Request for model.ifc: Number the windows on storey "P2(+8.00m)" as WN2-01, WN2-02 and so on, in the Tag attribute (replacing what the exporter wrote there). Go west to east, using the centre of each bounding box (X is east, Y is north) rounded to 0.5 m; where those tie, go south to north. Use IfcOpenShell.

First a look at what the model holds.

```python
import ifcopenshell
import ifcopenshell.util.element
import ifcopenshell.util.placement

model = ifcopenshell.open("model.ifc")
print(model.schema)
storey = next(s for s in model.by_type("IfcBuildingStorey") if s.Name == "P2(+8.00m)")
windows = [e for e in ifcopenshell.util.element.get_decomposition(storey) if e.is_a("IfcWindow")]
for e in sorted(windows, key=lambda e: e.id()):
    origin = ifcopenshell.util.placement.get_local_placement(e.ObjectPlacement)[:3, 3]
    print(e.id(), e.Tag, e.Name, origin.round(2) + 0.0, sep=" | ")
```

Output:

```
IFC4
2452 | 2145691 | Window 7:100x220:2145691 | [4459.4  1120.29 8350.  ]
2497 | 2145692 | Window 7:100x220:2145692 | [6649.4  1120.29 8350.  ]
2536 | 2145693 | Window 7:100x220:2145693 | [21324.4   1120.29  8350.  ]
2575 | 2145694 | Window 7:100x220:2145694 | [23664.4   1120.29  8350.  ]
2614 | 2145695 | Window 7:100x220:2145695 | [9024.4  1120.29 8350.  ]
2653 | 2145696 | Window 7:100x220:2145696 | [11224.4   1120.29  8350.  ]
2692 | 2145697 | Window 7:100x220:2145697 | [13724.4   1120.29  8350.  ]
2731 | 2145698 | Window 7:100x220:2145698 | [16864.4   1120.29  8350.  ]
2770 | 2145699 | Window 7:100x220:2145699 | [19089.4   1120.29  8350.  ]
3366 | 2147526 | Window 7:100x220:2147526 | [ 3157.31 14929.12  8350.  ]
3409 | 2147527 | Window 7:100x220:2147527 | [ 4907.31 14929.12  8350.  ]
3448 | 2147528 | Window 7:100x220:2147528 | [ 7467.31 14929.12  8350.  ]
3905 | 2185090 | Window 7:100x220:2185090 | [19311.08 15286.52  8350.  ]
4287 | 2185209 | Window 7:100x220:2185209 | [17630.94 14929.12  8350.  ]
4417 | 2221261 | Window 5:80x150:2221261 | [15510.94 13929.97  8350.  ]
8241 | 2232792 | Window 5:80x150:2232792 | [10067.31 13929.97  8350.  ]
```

```python
import ifcopenshell
import ifcopenshell.geom
import ifcopenshell.util.element
import ifcopenshell.util.shape

model = ifcopenshell.open("model.ifc")
settings = ifcopenshell.geom.settings()
settings.set("use-world-coords", True)


def centre(element):
    shape = ifcopenshell.geom.create_shape(settings, element)
    return ifcopenshell.util.shape.get_bbox_centroid(shape.geometry)


storey = next(s for s in model.by_type("IfcBuildingStorey") if s.Name == "P2(+8.00m)")
windows = [e for e in ifcopenshell.util.element.get_decomposition(storey) if e.is_a("IfcWindow")]

# Insertion points can sit at a corner or the storey origin, so sort by the geometry (in metres).
centres = {e: centre(e) for e in windows}
windows.sort(key=lambda e: (round(centres[e][0] / 0.5), centres[e][1]))

for i, e in enumerate(windows, start=1):
    number = f"WN2-{i:02d}"
    e.Tag = number
    print(e.id(), number)

model.write("model_updated.ifc")
```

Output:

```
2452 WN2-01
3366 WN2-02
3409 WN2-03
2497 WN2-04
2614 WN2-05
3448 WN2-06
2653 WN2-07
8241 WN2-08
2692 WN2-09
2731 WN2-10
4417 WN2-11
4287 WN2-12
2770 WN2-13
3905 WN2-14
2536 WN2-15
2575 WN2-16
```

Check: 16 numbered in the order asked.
